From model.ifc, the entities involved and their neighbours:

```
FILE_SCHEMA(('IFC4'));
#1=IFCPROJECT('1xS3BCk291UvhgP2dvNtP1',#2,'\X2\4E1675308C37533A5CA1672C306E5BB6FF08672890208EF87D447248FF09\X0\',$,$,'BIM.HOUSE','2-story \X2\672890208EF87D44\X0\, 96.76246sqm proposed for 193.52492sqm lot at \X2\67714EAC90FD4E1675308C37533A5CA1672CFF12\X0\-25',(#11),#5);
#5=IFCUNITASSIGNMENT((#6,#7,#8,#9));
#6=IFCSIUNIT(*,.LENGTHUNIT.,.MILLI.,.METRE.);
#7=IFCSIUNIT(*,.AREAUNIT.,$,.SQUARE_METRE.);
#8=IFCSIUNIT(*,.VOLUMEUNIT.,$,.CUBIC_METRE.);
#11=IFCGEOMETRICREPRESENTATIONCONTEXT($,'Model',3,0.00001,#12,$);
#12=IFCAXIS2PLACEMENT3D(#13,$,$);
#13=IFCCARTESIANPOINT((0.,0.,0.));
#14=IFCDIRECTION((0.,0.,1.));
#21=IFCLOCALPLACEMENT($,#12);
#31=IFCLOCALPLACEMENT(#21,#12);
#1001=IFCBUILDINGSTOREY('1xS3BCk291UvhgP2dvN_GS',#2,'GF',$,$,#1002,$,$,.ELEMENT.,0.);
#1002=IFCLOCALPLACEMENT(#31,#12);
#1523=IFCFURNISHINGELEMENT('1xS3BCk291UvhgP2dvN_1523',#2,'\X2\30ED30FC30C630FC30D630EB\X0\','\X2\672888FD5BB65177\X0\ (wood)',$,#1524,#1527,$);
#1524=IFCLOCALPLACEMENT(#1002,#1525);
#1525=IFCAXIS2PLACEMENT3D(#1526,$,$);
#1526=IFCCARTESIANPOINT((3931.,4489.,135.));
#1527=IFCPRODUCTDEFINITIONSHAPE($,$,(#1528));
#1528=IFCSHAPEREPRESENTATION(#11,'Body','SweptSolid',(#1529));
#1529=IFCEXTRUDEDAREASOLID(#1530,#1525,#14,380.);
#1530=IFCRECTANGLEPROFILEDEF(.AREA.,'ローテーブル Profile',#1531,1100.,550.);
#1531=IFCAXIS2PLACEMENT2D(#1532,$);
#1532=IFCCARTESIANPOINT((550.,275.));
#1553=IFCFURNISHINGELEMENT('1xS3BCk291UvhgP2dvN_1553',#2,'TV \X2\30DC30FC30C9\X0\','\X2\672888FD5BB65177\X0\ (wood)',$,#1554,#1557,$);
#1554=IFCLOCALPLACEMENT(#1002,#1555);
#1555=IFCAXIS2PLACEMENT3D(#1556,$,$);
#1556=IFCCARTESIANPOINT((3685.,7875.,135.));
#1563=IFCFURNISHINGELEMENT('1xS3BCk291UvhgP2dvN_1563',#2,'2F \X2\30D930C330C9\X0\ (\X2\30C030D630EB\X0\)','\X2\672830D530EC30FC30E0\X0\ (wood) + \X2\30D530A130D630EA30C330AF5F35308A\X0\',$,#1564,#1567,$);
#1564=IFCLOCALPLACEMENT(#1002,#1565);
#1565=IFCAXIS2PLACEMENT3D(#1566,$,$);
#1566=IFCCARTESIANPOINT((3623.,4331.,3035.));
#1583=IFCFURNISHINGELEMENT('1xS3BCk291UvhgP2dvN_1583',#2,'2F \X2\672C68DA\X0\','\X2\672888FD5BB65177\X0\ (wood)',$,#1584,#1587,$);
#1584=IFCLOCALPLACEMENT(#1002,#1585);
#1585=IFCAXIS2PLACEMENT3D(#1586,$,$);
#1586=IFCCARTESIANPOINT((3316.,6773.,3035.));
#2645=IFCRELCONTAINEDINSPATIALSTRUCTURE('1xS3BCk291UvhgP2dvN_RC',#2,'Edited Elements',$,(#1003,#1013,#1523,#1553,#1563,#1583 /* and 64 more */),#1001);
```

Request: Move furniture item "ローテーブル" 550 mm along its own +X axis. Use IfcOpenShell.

```python
import ifcopenshell
import ifcopenshell.api.geometry
import ifcopenshell.util.placement

model = ifcopenshell.open("model.ifc")

item = model.by_guid("1xS3BCk291UvhgP2dvN_1523")
matrix = ifcopenshell.util.placement.get_local_placement(item.ObjectPlacement)
matrix[:3, 3] += matrix[:3, 0] * 550.0
ifcopenshell.api.geometry.edit_object_placement(model, product=item, matrix=matrix, is_si=False)

print(ifcopenshell.util.placement.get_local_placement(item.ObjectPlacement).round(3) + 0.0)

model.write("model_updated.ifc")
```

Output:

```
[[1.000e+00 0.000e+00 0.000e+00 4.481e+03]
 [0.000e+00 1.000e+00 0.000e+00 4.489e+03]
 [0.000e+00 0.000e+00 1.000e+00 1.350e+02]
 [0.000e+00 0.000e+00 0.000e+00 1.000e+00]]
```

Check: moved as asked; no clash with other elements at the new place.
